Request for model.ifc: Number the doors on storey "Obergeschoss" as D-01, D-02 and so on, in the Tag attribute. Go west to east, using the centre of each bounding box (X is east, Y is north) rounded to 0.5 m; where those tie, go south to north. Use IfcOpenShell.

First a look at what the model holds.

```python
import ifcopenshell
import ifcopenshell.util.element
import ifcopenshell.util.placement

model = ifcopenshell.open("model.ifc")
print(model.schema)
storey = next(s for s in model.by_type("IfcBuildingStorey") if s.Name == "Obergeschoss")
doors = [e for e in ifcopenshell.util.element.get_decomposition(storey) if e.is_a("IfcDoor")]
for e in sorted(doors, key=lambda e: e.id()):
    origin = ifcopenshell.util.placement.get_local_placement(e.ObjectPlacement)[:3, 3]
    print(e.id(), e.Tag, e.Name, origin.round(2) + 0.0, sep=" | ")
```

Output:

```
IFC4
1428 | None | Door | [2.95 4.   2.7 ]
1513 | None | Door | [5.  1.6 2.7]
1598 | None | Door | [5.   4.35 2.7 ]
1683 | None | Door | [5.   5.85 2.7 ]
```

```python
import ifcopenshell
import ifcopenshell.geom
import ifcopenshell.util.element
import ifcopenshell.util.shape

model = ifcopenshell.open("model.ifc")
settings = ifcopenshell.geom.settings()
settings.set("use-world-coords", True)


def centre(element):
    shape = ifcopenshell.geom.create_shape(settings, element)
    return ifcopenshell.util.shape.get_bbox_centroid(shape.geometry)


storey = next(s for s in model.by_type("IfcBuildingStorey") if s.Name == "Obergeschoss")
doors = [e for e in ifcopenshell.util.element.get_decomposition(storey) if e.is_a("IfcDoor")]

# Insertion points can sit at a corner or the storey origin, so sort by the geometry (in metres).
centres = {e: centre(e) for e in doors}
doors.sort(key=lambda e: (round(centres[e][0] / 0.5), centres[e][1]))

for i, e in enumerate(doors, start=1):
    number = f"D-{i:02d}"
    e.Tag = number
    print(e.id(), number)

model.write("model_updated.ifc")
```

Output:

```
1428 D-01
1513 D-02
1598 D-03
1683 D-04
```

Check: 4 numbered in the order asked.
